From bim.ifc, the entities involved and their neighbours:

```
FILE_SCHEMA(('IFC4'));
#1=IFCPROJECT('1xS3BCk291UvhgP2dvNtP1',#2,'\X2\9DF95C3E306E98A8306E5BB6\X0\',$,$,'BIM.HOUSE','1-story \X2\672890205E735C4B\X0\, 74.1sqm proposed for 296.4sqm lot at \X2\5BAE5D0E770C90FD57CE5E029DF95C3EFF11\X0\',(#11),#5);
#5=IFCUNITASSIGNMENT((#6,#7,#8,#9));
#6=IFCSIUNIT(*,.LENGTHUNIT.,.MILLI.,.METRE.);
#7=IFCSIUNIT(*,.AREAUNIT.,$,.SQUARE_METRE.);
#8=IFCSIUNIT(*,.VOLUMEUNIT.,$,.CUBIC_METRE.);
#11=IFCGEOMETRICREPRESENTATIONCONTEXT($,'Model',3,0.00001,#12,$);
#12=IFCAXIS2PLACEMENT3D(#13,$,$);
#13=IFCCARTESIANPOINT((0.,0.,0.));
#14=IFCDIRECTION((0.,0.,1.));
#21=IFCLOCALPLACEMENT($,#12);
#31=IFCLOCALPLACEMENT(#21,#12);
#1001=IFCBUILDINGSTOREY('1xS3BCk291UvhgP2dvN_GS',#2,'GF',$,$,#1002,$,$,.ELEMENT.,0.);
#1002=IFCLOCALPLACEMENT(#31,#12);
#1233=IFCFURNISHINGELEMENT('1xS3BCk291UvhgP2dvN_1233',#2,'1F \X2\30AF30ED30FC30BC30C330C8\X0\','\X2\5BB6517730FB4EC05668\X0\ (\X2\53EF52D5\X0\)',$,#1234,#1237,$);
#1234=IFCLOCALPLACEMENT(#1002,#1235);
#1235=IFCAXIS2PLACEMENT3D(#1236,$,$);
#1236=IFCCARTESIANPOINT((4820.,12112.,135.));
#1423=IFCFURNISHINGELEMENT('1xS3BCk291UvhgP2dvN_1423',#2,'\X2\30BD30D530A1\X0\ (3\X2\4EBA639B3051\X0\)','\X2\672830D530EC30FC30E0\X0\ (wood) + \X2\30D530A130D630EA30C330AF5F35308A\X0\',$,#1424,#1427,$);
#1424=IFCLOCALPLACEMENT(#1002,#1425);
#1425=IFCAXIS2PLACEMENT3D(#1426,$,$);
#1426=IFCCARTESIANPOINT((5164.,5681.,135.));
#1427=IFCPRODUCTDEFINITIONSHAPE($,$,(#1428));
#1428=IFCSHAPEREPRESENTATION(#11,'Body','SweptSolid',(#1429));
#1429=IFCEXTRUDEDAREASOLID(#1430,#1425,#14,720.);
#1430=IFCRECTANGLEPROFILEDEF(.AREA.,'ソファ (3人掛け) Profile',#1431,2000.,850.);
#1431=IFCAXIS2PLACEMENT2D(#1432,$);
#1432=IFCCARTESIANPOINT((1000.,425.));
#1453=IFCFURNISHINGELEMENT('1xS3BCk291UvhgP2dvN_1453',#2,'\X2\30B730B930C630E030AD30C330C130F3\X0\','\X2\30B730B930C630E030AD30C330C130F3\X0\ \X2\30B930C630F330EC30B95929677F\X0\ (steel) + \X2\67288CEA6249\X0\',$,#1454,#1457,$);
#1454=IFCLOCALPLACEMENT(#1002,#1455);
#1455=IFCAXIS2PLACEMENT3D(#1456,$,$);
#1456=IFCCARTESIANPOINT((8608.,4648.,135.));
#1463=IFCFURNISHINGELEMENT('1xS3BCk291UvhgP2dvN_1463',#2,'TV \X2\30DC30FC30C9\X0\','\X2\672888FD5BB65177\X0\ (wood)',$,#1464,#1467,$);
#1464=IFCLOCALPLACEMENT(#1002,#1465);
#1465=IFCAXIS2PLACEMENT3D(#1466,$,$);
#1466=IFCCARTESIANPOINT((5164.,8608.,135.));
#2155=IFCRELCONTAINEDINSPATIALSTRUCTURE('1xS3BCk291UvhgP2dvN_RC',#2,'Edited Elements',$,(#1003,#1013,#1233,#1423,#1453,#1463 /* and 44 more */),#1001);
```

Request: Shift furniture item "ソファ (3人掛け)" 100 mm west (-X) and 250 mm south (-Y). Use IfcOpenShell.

```python
import ifcopenshell
import ifcopenshell.api.geometry
import ifcopenshell.util.placement

model = ifcopenshell.open("bim.ifc")

item = model.by_id(1423)
matrix = ifcopenshell.util.placement.get_local_placement(item.ObjectPlacement)
matrix[0, 3] -= 100.0
matrix[1, 3] -= 250.0
ifcopenshell.api.geometry.edit_object_placement(model, product=item, matrix=matrix, is_si=False)

print(ifcopenshell.util.placement.get_local_placement(item.ObjectPlacement).round(3) + 0.0)

model.write("bim_rev.ifc")
```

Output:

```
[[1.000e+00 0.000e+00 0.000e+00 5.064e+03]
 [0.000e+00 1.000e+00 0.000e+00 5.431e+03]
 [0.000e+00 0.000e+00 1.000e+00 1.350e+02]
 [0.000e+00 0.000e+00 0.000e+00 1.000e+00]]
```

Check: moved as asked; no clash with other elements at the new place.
